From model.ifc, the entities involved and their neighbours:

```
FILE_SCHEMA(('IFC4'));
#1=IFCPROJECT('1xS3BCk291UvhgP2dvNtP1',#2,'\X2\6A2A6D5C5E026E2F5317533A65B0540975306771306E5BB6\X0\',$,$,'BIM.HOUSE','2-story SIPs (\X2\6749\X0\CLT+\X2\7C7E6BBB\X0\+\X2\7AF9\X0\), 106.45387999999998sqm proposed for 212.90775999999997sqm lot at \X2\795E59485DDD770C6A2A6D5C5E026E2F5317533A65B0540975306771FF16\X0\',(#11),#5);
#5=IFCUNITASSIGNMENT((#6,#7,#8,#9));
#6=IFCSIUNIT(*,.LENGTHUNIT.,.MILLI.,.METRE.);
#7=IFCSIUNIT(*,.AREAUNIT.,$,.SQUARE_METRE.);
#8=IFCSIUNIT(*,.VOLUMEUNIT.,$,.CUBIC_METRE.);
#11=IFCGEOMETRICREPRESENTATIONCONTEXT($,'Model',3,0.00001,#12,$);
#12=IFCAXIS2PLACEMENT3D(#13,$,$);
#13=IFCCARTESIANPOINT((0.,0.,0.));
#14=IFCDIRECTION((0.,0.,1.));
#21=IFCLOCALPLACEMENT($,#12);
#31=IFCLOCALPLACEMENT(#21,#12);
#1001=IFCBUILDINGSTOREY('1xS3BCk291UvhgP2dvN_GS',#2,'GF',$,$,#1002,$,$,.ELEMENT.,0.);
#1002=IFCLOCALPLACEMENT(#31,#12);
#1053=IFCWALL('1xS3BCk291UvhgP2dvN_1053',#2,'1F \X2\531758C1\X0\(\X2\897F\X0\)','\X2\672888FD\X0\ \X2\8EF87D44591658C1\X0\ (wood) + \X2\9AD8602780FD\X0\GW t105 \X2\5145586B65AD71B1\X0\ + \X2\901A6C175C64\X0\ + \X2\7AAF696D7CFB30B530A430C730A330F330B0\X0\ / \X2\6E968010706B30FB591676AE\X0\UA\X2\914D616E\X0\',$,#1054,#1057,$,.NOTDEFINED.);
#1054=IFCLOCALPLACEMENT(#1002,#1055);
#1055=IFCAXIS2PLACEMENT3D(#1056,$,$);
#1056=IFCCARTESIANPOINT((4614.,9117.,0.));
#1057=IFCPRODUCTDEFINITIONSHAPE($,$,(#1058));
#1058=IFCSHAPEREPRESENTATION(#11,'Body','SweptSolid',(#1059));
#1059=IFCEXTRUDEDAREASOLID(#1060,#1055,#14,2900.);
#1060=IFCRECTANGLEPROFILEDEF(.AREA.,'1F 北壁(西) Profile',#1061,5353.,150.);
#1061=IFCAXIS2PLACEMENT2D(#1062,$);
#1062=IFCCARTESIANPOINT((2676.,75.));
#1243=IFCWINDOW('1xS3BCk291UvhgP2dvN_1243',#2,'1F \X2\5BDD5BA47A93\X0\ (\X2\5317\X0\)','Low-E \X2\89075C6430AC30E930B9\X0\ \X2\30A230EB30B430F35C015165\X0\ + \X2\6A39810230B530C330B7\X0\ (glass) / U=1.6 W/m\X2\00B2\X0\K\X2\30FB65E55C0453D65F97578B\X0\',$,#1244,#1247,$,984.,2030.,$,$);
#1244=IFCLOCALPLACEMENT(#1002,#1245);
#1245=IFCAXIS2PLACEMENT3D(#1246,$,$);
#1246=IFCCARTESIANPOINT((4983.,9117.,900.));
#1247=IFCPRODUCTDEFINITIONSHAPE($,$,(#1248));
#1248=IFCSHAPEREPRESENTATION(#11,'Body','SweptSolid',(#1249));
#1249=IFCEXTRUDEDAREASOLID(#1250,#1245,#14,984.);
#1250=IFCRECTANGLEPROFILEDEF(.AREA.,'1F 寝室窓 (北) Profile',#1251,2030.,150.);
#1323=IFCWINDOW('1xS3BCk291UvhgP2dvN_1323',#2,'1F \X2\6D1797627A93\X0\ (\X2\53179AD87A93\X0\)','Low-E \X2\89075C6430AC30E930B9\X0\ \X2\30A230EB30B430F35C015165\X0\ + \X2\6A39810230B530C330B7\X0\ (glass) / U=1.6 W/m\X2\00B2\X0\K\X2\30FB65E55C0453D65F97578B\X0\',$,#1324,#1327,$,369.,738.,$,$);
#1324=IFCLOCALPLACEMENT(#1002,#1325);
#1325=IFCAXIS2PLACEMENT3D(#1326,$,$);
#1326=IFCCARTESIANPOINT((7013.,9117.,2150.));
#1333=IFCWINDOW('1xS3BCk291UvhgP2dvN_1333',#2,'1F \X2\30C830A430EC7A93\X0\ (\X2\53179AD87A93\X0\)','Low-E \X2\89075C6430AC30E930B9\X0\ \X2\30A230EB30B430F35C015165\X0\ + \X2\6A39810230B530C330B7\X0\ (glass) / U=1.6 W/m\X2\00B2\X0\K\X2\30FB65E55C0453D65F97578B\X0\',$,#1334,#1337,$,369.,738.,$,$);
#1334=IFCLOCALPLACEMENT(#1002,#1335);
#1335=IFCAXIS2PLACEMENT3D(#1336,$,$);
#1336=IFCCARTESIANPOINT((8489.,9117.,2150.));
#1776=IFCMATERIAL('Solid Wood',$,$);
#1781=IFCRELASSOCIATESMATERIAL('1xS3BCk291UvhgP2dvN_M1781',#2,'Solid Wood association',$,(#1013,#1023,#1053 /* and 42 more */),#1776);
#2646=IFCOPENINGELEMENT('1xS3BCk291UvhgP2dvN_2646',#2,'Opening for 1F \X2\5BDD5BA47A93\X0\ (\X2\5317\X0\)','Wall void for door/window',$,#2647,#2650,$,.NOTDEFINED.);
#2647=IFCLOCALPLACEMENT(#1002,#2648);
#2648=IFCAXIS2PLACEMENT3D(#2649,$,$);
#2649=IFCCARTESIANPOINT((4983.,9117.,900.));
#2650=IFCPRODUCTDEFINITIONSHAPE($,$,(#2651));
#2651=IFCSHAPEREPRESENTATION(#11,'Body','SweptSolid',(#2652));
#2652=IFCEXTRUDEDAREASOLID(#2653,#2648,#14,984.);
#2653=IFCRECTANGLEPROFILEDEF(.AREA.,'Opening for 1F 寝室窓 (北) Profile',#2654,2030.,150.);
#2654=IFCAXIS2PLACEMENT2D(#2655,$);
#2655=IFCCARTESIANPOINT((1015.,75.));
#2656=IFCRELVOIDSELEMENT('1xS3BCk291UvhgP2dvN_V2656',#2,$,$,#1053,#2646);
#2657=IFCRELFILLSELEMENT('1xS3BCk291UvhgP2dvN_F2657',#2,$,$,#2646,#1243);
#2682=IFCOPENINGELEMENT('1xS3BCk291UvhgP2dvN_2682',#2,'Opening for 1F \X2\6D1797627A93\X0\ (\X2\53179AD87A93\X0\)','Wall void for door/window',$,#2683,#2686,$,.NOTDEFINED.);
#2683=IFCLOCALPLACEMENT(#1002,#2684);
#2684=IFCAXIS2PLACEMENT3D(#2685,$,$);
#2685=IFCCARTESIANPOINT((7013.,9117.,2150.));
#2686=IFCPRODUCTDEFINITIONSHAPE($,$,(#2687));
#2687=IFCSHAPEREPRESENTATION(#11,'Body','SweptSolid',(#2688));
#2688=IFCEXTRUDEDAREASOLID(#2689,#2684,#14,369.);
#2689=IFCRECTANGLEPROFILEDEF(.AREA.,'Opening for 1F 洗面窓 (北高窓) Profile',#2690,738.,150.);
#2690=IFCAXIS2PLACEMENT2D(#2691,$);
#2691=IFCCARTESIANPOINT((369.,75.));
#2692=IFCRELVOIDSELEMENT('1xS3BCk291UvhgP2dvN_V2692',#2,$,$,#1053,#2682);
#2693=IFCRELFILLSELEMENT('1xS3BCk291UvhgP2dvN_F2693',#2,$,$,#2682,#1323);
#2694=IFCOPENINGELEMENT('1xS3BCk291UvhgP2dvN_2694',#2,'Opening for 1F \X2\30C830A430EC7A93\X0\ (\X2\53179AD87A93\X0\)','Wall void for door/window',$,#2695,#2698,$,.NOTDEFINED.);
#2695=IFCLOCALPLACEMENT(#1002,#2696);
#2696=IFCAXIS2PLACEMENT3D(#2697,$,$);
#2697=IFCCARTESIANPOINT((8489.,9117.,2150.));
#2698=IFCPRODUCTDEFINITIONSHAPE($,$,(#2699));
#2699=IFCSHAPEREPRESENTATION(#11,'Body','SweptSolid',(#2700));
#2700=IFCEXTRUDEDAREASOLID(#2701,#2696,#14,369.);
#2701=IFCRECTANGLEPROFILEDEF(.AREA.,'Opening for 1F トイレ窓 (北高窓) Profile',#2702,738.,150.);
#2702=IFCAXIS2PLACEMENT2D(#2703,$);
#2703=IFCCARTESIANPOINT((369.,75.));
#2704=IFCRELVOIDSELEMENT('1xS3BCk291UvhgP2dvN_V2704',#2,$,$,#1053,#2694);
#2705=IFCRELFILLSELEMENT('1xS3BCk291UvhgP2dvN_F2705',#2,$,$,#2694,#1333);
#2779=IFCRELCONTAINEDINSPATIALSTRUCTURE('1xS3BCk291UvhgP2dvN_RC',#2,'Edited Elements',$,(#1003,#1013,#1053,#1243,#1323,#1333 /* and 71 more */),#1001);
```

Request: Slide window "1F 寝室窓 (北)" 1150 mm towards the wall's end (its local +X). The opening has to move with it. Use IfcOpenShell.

```python
import ifcopenshell
import ifcopenshell.api.geometry
import ifcopenshell.util.placement

model = ifcopenshell.open("model.ifc")

window = model.by_guid("1xS3BCk291UvhgP2dvN_1243")
opening = window.FillsVoids[0].RelatingOpeningElement
wall = opening.VoidsElements[0].RelatingBuildingElement

wall_matrix = ifcopenshell.util.placement.get_local_placement(wall.ObjectPlacement)
shift = wall_matrix[:3, 0] * 1150.0
before = ifcopenshell.util.placement.get_local_placement(window.ObjectPlacement)[:3, 3].copy()

# The window is not placed relative to its opening, so move both.
for product in (opening, window):
    matrix = ifcopenshell.util.placement.get_local_placement(product.ObjectPlacement)
    matrix[:3, 3] += shift
    ifcopenshell.api.geometry.edit_object_placement(model, product=product, matrix=matrix, is_si=False)

after = ifcopenshell.util.placement.get_local_placement(window.ObjectPlacement)[:3, 3]
print("window moved by", (after - before).round(3) + 0.0)

model.write("model_edited.ifc")
```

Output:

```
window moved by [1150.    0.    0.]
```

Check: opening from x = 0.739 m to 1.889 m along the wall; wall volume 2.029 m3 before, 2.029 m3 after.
